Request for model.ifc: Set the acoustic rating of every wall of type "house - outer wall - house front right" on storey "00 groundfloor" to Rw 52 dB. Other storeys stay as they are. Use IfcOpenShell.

First a look at what the model holds.

```python
import ifcopenshell
import ifcopenshell.util.element

model = ifcopenshell.open("model.ifc")
print(model.schema)
storey = next(s for s in model.by_type("IfcBuildingStorey") if s.Name == "00 groundfloor")
walls = [e for e in ifcopenshell.util.element.get_decomposition(storey) if e.is_a("IfcWall")]
seen = {}
for e in walls:
    element_type = ifcopenshell.util.element.get_type(e)
    key = (element_type.Name if element_type != e and element_type else None, ifcopenshell.util.element.get_pset(e, "Pset_WallCommon", "AcousticRating"))
    seen[key] = seen.get(key, 0) + 1
for (name, value), count in sorted(seen.items(), key=str):
    print(count, "x", name, "|", value)
```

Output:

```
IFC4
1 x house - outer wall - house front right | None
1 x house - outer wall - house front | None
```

```python
import ifcopenshell
import ifcopenshell.api.pset
import ifcopenshell.util.element

model = ifcopenshell.open("model.ifc")

storey = next(s for s in model.by_type("IfcBuildingStorey") if s.Name == "00 groundfloor")
walls = [e for e in ifcopenshell.util.element.get_decomposition(storey) if e.is_a("IfcWall")]

count = 0
for e in walls:
    element_type = ifcopenshell.util.element.get_type(e)
    if element_type in (None, e) or element_type.Name != "house - outer wall - house front right":
        continue
    # add_pset returns the element's existing set when there is one.
    pset = ifcopenshell.api.pset.add_pset(model, product=e, name="Pset_WallCommon")
    ifcopenshell.api.pset.edit_pset(model, pset=pset, properties={"AcousticRating": "Rw 52 dB"})
    count += 1

print(count, "walls updated")

model.write("model_edited.ifc")
```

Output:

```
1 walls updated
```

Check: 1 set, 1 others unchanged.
